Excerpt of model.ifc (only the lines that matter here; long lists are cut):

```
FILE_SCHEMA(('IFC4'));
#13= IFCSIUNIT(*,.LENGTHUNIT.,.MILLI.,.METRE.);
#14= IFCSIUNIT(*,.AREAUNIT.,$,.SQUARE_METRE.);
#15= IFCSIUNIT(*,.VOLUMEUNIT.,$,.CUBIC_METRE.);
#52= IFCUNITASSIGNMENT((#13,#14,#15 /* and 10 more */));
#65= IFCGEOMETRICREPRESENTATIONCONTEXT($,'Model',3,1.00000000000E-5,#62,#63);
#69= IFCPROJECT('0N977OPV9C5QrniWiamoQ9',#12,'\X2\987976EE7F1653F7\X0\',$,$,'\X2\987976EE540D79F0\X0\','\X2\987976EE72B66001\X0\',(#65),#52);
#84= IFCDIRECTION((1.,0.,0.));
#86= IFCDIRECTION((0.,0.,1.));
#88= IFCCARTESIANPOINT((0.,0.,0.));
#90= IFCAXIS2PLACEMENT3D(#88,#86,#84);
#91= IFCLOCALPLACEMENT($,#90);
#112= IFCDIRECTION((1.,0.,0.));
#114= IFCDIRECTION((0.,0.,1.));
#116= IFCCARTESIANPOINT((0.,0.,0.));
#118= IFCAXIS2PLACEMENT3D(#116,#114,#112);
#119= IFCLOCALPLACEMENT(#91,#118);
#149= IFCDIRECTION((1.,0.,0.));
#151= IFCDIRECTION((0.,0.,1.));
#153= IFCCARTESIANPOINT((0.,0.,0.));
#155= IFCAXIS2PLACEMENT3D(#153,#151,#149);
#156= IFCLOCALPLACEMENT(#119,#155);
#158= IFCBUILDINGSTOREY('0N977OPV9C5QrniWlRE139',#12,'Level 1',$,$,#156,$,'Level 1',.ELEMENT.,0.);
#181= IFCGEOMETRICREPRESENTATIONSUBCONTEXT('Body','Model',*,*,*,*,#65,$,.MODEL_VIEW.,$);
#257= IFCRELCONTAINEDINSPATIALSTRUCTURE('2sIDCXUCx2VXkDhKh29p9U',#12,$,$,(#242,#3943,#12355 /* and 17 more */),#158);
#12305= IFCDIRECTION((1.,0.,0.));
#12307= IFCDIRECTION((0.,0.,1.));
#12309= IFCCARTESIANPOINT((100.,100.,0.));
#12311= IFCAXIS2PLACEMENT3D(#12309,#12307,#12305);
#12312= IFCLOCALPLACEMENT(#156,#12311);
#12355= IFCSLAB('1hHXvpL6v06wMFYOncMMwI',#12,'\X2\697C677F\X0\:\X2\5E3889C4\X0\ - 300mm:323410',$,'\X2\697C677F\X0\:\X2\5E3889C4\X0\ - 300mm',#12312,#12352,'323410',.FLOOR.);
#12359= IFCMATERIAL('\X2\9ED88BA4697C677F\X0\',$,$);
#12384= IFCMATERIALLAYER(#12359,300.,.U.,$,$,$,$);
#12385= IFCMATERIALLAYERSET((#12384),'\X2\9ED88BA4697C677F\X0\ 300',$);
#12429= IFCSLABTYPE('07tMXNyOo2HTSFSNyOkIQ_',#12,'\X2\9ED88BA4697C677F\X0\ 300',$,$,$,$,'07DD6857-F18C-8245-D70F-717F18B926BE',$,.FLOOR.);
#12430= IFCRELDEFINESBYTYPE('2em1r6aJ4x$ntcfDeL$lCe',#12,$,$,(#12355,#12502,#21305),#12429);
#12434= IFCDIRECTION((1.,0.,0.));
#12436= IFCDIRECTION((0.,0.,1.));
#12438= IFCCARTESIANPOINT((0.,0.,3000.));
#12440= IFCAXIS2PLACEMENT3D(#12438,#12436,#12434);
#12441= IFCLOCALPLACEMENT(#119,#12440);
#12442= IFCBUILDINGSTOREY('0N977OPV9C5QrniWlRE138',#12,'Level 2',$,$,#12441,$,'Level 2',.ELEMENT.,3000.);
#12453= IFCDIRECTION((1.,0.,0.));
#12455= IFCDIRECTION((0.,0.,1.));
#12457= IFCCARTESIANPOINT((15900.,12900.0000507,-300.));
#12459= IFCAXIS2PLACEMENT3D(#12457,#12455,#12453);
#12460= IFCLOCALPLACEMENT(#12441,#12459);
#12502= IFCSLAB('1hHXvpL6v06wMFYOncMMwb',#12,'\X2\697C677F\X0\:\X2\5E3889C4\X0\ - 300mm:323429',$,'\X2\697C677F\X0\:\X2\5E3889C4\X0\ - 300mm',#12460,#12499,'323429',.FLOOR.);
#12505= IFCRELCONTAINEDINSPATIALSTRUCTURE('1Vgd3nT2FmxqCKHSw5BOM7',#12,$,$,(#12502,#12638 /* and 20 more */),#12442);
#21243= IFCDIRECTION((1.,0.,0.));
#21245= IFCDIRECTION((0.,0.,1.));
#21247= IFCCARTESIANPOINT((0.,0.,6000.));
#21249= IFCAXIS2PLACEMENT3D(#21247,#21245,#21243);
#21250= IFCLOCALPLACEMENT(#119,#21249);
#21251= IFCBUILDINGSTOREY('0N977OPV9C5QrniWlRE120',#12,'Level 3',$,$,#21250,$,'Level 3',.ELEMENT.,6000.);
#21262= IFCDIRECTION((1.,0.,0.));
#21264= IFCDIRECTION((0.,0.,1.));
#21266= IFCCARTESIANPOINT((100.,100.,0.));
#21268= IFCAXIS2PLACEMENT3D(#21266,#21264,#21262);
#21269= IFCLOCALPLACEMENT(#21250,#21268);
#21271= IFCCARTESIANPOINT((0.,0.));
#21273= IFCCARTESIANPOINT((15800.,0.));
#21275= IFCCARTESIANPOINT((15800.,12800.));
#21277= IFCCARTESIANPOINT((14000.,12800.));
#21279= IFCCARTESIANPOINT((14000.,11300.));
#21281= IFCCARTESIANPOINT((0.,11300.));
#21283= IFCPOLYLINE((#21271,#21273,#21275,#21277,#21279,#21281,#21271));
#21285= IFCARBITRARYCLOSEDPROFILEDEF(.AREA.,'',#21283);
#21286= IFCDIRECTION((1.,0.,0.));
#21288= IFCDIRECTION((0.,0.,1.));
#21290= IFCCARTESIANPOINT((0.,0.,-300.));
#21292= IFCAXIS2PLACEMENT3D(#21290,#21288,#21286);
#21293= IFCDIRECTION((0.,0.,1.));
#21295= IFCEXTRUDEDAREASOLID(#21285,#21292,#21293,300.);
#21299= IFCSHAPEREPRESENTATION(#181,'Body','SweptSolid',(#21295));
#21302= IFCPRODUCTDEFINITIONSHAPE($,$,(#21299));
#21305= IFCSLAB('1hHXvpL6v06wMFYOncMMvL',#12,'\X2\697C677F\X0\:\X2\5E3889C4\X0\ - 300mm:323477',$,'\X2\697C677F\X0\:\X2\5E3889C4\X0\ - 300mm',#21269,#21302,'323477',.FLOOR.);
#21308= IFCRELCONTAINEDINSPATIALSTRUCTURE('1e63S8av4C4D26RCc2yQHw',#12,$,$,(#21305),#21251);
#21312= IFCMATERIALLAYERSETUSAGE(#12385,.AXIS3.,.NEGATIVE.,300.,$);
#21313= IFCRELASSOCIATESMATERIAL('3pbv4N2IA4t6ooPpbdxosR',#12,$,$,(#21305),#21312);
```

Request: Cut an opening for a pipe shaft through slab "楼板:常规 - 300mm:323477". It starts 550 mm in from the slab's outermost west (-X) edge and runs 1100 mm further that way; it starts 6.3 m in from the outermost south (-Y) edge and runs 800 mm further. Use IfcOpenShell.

```python
import numpy as np
import ifcopenshell
import ifcopenshell.api.feature
import ifcopenshell.api.geometry
import ifcopenshell.api.root
import ifcopenshell.geom
import ifcopenshell.util.placement
import ifcopenshell.util.representation
import ifcopenshell.util.shape
import ifcopenshell.util.unit

model = ifcopenshell.open("model.ifc")
unit_scale = ifcopenshell.util.unit.calculate_unit_scale(model)
settings = ifcopenshell.geom.settings()


def volume(element):
    """Net volume in cubic metres, openings subtracted."""
    shape = ifcopenshell.geom.create_shape(settings, element)
    return ifcopenshell.util.shape.get_volume(shape.geometry)


slab = model.by_id(21305)
before = volume(slab)

# Extent in the slab's own axes, in metres. The edges named are its -X and -Y sides.
slab_shape = ifcopenshell.geom.create_shape(settings, slab)
vertices = ifcopenshell.util.shape.get_vertices(slab_shape.geometry)
x_min, y_min, bottom = vertices.min(axis=0)
top = vertices[:, 2].max()

opening = ifcopenshell.api.root.create_entity(model, ifc_class="IfcOpeningElement", name="Pipe shaft opening", predefined_type="OPENING")
context = ifcopenshell.util.representation.get_context(model, "Model", "Body", "MODEL_VIEW")
width, depth = 1.1, 0.8
outline = [(0.0, 0.0), (width, 0.0), (width, depth), (0.0, depth), (0.0, 0.0)]
# Overshoot both faces by 50 mm so the cut is clean.
shape = ifcopenshell.api.geometry.add_slab_representation(
    model, context=context, depth=top - bottom + 0.1, polyline=outline
)
ifcopenshell.api.geometry.assign_representation(model, product=opening, representation=shape)

matrix = ifcopenshell.util.placement.get_local_placement(slab.ObjectPlacement)
matrix[:, 3] = matrix @ np.append(np.array([x_min + 0.55, y_min + 6.3, bottom - 0.05]) / unit_scale, 1.0)
ifcopenshell.api.geometry.edit_object_placement(model, product=opening, matrix=matrix, is_si=False)
ifcopenshell.api.feature.add_feature(model, feature=opening, element=slab)

after = volume(slab)

print(f"slab volume {before:.3f} -> {after:.3f} m3")

model.write("model-out.ifc")
```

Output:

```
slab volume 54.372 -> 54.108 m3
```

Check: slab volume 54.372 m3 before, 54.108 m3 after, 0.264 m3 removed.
